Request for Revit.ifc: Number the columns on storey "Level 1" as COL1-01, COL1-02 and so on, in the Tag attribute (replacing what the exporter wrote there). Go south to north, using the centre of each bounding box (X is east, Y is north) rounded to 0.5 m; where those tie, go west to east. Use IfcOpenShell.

First a look at what the model holds.

```python
import ifcopenshell
import ifcopenshell.util.element
import ifcopenshell.util.placement

model = ifcopenshell.open("Revit.ifc")
print(model.schema)
storey = next(s for s in model.by_type("IfcBuildingStorey") if s.Name == "Level 1")
columns = [e for e in ifcopenshell.util.element.get_decomposition(storey) if e.is_a("IfcColumn")]
for e in sorted(columns, key=lambda e: e.id()):
    origin = ifcopenshell.util.placement.get_local_placement(e.ObjectPlacement)[:3, 3]
    print(e.id(), e.Tag, e.Name, origin.round(2) + 0.0, sep=" | ")
```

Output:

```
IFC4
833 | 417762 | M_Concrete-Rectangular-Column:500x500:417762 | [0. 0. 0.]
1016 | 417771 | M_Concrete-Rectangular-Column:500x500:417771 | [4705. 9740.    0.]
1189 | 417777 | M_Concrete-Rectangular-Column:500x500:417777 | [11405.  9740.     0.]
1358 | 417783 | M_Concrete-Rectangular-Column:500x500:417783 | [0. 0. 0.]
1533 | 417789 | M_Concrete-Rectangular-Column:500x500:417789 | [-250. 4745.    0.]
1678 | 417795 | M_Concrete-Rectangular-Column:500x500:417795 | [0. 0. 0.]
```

```python
import ifcopenshell
import ifcopenshell.geom
import ifcopenshell.util.element
import ifcopenshell.util.shape

model = ifcopenshell.open("Revit.ifc")
settings = ifcopenshell.geom.settings()
settings.set("use-world-coords", True)


def centre(element):
    shape = ifcopenshell.geom.create_shape(settings, element)
    return ifcopenshell.util.shape.get_bbox_centroid(shape.geometry)


storey = next(s for s in model.by_type("IfcBuildingStorey") if s.Name == "Level 1")
columns = [e for e in ifcopenshell.util.element.get_decomposition(storey) if e.is_a("IfcColumn")]

# Insertion points can sit at a corner or the storey origin, so sort by the geometry (in metres).
centres = {e: centre(e) for e in columns}
columns.sort(key=lambda e: (round(centres[e][1] / 0.5), centres[e][0]))

for i, e in enumerate(columns, start=1):
    number = f"COL1-{i:02d}"
    e.Tag = number
    print(e.id(), number)

model.write("Revit_rev.ifc")
```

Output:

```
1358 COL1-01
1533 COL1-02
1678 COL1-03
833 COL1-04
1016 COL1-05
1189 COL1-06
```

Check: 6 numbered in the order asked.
